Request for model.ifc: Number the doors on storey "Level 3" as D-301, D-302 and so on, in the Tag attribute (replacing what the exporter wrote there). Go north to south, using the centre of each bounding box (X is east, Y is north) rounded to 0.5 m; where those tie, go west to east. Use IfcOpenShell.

First a look at what the model holds.

```python
import ifcopenshell
import ifcopenshell.util.element
import ifcopenshell.util.placement

model = ifcopenshell.open("model.ifc")
print(model.schema)
storey = next(s for s in model.by_type("IfcBuildingStorey") if s.Name == "Level 3")
doors = [e for e in ifcopenshell.util.element.get_decomposition(storey) if e.is_a("IfcDoor")]
for e in sorted(doors, key=lambda e: e.id()):
    origin = ifcopenshell.util.placement.get_local_placement(e.ObjectPlacement)[:3, 3]
    print(e.id(), e.Tag, e.Name, origin.round(2) + 0.0, sep=" | ")
```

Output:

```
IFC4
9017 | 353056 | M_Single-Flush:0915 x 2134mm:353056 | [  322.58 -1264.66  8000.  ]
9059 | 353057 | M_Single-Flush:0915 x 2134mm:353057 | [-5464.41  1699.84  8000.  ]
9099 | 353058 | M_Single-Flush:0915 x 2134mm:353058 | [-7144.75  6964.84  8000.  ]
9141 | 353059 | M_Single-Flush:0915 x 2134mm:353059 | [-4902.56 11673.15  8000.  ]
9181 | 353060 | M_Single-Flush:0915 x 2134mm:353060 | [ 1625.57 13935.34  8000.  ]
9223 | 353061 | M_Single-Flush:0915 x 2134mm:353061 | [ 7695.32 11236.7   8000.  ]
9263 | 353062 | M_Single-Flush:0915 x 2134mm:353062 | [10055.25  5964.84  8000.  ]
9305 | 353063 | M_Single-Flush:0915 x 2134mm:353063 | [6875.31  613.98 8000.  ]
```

```python
import ifcopenshell
import ifcopenshell.geom
import ifcopenshell.util.element
import ifcopenshell.util.shape

model = ifcopenshell.open("model.ifc")
settings = ifcopenshell.geom.settings()
settings.set("use-world-coords", True)


def centre(element):
    shape = ifcopenshell.geom.create_shape(settings, element)
    return ifcopenshell.util.shape.get_bbox_centroid(shape.geometry)


storey = next(s for s in model.by_type("IfcBuildingStorey") if s.Name == "Level 3")
doors = [e for e in ifcopenshell.util.element.get_decomposition(storey) if e.is_a("IfcDoor")]

# Insertion points can sit at a corner or the storey origin, so sort by the geometry (in metres).
centres = {e: centre(e) for e in doors}
doors.sort(key=lambda e: (-round(centres[e][1] / 0.5), centres[e][0]))

for i, e in enumerate(doors, start=1):
    number = f"D-3{i:02d}"
    e.Tag = number
    print(e.id(), number)

model.write("model_v2.ifc")
```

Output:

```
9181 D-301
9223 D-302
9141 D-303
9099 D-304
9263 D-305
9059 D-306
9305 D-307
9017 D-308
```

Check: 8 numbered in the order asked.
